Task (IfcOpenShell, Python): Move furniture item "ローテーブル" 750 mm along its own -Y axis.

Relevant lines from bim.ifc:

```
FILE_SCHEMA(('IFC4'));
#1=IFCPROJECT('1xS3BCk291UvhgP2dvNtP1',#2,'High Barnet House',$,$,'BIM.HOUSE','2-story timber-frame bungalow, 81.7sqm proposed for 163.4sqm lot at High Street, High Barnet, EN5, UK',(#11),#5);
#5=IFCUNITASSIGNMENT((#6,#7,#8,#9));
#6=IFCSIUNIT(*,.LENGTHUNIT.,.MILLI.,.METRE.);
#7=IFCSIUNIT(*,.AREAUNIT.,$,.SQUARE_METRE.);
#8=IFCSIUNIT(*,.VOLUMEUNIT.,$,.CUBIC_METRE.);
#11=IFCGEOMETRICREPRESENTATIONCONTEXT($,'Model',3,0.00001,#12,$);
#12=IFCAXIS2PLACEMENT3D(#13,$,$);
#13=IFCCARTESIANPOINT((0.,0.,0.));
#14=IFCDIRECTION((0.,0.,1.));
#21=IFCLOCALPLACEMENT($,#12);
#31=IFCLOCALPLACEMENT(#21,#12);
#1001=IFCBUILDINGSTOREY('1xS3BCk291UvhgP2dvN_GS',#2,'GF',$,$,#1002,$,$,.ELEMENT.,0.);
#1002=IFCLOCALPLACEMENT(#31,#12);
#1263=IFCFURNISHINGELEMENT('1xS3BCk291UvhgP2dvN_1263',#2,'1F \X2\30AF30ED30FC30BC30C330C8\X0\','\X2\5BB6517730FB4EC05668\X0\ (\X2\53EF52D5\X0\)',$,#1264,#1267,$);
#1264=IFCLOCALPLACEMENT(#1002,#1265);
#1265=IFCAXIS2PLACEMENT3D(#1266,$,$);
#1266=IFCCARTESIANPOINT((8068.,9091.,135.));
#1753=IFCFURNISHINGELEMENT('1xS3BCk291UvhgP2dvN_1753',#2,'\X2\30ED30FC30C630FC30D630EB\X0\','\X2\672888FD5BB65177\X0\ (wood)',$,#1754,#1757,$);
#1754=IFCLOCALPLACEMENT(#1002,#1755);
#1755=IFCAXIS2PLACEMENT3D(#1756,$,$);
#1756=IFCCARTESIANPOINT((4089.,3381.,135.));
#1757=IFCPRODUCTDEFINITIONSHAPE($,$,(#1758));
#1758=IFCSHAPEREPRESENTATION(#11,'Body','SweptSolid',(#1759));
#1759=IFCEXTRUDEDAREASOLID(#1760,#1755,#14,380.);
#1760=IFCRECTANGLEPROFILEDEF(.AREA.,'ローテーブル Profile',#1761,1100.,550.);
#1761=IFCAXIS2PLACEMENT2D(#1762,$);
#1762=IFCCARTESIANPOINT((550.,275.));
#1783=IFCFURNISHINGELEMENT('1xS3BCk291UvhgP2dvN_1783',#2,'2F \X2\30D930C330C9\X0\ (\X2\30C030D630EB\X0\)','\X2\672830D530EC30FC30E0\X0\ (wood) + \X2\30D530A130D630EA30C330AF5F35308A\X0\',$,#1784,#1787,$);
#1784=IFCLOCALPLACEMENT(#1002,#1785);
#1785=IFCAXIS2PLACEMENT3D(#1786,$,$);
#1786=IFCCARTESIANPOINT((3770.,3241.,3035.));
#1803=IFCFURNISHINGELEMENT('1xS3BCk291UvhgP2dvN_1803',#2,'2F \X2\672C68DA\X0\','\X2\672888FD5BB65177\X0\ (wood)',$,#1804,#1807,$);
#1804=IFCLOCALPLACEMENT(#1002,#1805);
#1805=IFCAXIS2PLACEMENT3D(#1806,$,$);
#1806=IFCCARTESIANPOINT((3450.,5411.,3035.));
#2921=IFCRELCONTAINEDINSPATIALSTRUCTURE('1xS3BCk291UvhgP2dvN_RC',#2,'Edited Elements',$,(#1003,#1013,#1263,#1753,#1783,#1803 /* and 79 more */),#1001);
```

```python
import ifcopenshell
import ifcopenshell.api.geometry
import ifcopenshell.util.placement

model = ifcopenshell.open("bim.ifc")

item = model.by_guid("1xS3BCk291UvhgP2dvN_1753")
matrix = ifcopenshell.util.placement.get_local_placement(item.ObjectPlacement)
matrix[:3, 3] -= matrix[:3, 1] * 750.0
ifcopenshell.api.geometry.edit_object_placement(model, product=item, matrix=matrix, is_si=False)

print(ifcopenshell.util.placement.get_local_placement(item.ObjectPlacement).round(3) + 0.0)

model.write("bim_rev.ifc")
```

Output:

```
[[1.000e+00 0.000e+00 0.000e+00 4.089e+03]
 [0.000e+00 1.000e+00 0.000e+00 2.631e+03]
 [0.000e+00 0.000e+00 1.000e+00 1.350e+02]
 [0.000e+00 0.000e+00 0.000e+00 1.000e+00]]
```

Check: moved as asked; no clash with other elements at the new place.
